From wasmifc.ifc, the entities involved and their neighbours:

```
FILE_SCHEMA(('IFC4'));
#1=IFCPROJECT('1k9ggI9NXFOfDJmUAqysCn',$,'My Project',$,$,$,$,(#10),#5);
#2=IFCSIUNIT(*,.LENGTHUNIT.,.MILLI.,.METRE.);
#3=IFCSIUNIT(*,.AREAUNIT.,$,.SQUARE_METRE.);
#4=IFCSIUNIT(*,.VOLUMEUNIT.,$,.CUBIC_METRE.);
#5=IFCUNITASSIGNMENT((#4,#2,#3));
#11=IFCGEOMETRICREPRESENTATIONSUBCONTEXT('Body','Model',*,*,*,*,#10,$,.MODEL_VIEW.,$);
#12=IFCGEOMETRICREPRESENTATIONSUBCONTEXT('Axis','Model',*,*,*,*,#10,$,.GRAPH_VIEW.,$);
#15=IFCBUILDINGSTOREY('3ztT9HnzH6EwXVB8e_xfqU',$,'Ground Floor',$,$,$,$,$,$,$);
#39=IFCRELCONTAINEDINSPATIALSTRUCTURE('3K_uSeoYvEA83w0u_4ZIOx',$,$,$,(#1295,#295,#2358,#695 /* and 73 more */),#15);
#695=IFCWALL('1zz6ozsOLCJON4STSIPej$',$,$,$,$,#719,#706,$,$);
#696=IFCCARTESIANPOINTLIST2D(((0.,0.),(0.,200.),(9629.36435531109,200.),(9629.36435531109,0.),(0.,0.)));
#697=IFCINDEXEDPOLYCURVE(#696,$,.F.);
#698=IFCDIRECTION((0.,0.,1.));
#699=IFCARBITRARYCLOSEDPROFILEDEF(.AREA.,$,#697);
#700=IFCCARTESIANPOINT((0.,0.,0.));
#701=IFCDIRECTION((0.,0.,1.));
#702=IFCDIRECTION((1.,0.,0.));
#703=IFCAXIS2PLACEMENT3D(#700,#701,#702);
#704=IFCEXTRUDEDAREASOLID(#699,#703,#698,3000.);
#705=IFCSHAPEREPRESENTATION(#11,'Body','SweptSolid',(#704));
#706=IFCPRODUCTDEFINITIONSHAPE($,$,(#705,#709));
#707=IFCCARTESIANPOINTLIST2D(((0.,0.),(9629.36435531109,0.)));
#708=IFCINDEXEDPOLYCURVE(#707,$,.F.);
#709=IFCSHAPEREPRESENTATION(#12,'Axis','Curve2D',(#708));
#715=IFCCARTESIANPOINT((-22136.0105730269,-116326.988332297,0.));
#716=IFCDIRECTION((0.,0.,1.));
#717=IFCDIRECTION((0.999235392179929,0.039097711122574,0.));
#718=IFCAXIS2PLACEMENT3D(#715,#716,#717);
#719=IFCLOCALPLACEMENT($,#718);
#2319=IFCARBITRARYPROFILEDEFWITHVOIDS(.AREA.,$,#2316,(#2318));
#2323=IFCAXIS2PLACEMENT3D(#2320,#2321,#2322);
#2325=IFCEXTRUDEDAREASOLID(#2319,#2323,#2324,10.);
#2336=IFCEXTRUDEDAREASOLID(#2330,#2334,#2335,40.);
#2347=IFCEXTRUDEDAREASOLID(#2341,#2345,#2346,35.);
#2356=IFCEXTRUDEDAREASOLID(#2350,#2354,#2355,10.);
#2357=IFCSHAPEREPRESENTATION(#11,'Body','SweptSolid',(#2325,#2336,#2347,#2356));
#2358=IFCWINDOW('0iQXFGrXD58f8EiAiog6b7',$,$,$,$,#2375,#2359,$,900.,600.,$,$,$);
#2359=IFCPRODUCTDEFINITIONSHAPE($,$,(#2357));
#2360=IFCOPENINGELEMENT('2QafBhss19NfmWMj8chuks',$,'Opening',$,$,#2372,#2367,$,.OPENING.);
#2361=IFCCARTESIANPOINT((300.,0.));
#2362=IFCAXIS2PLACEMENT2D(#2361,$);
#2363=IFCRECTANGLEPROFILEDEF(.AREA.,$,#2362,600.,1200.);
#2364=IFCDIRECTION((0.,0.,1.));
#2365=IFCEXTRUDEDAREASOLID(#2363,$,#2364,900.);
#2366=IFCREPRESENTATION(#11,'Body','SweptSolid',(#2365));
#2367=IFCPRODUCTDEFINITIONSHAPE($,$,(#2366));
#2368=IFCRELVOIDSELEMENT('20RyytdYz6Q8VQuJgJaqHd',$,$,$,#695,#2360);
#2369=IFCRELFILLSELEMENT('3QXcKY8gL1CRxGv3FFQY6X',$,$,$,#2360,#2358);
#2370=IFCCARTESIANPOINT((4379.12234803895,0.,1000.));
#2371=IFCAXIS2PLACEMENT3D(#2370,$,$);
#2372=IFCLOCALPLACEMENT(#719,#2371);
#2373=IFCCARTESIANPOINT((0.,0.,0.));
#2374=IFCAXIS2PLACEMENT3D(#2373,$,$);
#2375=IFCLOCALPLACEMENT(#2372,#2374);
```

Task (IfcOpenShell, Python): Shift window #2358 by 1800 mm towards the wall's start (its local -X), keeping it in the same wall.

```python
import ifcopenshell
import ifcopenshell.api.geometry
import ifcopenshell.util.placement

model = ifcopenshell.open("wasmifc.ifc")

window = model.by_guid("0iQXFGrXD58f8EiAiog6b7")
opening = window.FillsVoids[0].RelatingOpeningElement
wall = opening.VoidsElements[0].RelatingBuildingElement

wall_matrix = ifcopenshell.util.placement.get_local_placement(wall.ObjectPlacement)
shift = wall_matrix[:3, 0] * -1800.0
before = ifcopenshell.util.placement.get_local_placement(window.ObjectPlacement)[:3, 3].copy()

# The window is placed relative to its opening, so it follows when the opening moves.
matrix = ifcopenshell.util.placement.get_local_placement(opening.ObjectPlacement)
matrix[:3, 3] += shift
ifcopenshell.api.geometry.edit_object_placement(
    model, product=opening, matrix=matrix, is_si=False, should_transform_children=True
)

after = ifcopenshell.util.placement.get_local_placement(window.ObjectPlacement)[:3, 3]
print("window moved by", (after - before).round(3) + 0.0)

model.write("wasmifc_rev.ifc")
```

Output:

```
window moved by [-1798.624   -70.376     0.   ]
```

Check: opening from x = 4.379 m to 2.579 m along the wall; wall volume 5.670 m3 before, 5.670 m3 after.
